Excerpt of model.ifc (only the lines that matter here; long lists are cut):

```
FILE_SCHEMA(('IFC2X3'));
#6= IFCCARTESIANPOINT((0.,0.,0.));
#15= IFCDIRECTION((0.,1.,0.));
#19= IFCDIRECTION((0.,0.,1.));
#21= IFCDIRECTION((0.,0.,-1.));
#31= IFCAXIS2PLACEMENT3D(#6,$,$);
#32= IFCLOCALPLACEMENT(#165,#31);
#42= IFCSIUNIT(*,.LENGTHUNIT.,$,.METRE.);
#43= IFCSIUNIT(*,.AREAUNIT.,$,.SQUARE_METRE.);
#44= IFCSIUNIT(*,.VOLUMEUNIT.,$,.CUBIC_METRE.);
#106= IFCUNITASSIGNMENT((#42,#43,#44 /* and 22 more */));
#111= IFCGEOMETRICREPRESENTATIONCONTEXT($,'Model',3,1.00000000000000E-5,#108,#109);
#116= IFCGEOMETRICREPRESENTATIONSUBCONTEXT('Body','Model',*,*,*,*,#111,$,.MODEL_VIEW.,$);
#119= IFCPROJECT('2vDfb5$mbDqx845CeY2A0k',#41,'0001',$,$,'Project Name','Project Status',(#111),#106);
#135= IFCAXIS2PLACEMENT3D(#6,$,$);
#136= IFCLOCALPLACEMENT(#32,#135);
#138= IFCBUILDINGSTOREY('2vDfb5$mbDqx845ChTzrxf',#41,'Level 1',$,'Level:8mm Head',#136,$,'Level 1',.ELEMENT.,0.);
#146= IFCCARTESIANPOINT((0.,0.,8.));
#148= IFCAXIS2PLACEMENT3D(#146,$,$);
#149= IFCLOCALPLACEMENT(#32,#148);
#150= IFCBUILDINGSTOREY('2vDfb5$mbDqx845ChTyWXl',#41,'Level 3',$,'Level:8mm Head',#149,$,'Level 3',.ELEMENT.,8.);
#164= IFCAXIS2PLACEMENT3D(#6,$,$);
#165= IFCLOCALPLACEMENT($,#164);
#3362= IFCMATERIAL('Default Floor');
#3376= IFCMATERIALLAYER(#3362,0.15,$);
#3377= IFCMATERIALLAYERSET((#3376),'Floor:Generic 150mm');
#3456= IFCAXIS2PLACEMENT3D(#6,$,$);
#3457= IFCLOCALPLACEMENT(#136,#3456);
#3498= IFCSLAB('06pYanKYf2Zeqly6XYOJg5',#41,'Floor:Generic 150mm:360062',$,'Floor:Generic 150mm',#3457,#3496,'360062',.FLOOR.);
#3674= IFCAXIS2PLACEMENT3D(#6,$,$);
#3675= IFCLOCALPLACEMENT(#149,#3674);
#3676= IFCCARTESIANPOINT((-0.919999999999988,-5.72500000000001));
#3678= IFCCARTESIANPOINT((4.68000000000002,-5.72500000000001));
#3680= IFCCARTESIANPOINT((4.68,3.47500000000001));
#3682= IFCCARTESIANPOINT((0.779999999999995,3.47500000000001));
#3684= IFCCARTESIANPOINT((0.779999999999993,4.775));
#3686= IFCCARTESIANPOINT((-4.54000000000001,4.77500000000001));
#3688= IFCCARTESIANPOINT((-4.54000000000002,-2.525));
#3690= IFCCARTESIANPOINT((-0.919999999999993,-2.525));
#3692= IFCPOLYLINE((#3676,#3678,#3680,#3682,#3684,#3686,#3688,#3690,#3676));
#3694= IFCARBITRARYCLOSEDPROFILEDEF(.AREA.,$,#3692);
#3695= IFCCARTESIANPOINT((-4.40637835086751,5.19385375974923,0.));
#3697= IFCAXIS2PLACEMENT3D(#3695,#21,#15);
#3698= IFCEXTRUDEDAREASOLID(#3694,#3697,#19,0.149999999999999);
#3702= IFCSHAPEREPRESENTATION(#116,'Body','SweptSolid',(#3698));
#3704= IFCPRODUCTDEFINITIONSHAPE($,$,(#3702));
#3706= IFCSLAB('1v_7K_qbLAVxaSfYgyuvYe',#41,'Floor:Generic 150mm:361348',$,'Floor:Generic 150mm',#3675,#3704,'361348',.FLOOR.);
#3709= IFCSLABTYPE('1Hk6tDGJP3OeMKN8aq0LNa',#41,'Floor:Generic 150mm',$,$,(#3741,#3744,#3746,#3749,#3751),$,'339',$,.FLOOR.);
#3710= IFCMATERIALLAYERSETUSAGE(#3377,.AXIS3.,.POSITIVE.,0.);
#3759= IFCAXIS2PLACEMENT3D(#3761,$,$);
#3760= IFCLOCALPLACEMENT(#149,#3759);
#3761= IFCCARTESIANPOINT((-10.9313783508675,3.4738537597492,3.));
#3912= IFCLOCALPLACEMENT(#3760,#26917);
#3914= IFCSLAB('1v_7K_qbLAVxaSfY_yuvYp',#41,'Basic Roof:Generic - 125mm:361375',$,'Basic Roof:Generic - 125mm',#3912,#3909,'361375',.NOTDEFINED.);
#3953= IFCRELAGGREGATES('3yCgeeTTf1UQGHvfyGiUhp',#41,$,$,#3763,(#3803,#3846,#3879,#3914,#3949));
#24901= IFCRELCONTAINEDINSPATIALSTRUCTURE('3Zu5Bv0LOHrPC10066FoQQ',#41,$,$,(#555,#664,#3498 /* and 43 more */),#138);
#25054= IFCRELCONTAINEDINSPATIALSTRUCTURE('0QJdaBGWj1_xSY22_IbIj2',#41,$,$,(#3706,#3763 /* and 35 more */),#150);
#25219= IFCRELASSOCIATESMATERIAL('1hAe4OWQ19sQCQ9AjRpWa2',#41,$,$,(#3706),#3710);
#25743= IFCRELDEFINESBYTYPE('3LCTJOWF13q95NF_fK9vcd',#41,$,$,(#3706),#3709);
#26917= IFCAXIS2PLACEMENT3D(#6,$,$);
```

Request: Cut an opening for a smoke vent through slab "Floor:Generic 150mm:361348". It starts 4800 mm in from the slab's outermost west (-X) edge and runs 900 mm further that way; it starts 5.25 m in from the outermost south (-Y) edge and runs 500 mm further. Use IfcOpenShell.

```python
import numpy as np
import ifcopenshell
import ifcopenshell.api.feature
import ifcopenshell.api.geometry
import ifcopenshell.api.root
import ifcopenshell.geom
import ifcopenshell.util.placement
import ifcopenshell.util.representation
import ifcopenshell.util.shape
import ifcopenshell.util.unit

model = ifcopenshell.open("model.ifc")
unit_scale = ifcopenshell.util.unit.calculate_unit_scale(model)
settings = ifcopenshell.geom.settings()


def volume(element):
    """Net volume in cubic metres, openings subtracted."""
    shape = ifcopenshell.geom.create_shape(settings, element)
    return ifcopenshell.util.shape.get_volume(shape.geometry)


slab = model.by_id(3706)
before = volume(slab)

# Extent in the slab's own axes, in metres. The edges named are its -X and -Y sides.
slab_shape = ifcopenshell.geom.create_shape(settings, slab)
vertices = ifcopenshell.util.shape.get_vertices(slab_shape.geometry)
x_min, y_min, bottom = vertices.min(axis=0)
top = vertices[:, 2].max()

opening = ifcopenshell.api.root.create_entity(model, ifc_class="IfcOpeningElement", name="Smoke vent opening")
context = ifcopenshell.util.representation.get_context(model, "Model", "Body", "MODEL_VIEW")
width, depth = 0.9, 0.5
outline = [(0.0, 0.0), (width, 0.0), (width, depth), (0.0, depth), (0.0, 0.0)]
# Overshoot both faces by 50 mm so the cut is clean.
shape = ifcopenshell.api.geometry.add_slab_representation(
    model, context=context, depth=top - bottom + 0.1, polyline=outline
)
ifcopenshell.api.geometry.assign_representation(model, product=opening, representation=shape)

matrix = ifcopenshell.util.placement.get_local_placement(slab.ObjectPlacement)
matrix[:, 3] = matrix @ np.append(np.array([x_min + 4.8, y_min + 5.25, bottom - 0.05]) / unit_scale, 1.0)
ifcopenshell.api.geometry.edit_object_placement(model, product=opening, matrix=matrix, is_si=False)
ifcopenshell.api.feature.add_feature(model, feature=opening, element=slab)

after = volume(slab)

print(f"slab volume {before:.3f} -> {after:.3f} m3")

model.write("model_rev.ifc")
```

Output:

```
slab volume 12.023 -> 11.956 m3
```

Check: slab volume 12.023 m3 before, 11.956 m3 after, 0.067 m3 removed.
